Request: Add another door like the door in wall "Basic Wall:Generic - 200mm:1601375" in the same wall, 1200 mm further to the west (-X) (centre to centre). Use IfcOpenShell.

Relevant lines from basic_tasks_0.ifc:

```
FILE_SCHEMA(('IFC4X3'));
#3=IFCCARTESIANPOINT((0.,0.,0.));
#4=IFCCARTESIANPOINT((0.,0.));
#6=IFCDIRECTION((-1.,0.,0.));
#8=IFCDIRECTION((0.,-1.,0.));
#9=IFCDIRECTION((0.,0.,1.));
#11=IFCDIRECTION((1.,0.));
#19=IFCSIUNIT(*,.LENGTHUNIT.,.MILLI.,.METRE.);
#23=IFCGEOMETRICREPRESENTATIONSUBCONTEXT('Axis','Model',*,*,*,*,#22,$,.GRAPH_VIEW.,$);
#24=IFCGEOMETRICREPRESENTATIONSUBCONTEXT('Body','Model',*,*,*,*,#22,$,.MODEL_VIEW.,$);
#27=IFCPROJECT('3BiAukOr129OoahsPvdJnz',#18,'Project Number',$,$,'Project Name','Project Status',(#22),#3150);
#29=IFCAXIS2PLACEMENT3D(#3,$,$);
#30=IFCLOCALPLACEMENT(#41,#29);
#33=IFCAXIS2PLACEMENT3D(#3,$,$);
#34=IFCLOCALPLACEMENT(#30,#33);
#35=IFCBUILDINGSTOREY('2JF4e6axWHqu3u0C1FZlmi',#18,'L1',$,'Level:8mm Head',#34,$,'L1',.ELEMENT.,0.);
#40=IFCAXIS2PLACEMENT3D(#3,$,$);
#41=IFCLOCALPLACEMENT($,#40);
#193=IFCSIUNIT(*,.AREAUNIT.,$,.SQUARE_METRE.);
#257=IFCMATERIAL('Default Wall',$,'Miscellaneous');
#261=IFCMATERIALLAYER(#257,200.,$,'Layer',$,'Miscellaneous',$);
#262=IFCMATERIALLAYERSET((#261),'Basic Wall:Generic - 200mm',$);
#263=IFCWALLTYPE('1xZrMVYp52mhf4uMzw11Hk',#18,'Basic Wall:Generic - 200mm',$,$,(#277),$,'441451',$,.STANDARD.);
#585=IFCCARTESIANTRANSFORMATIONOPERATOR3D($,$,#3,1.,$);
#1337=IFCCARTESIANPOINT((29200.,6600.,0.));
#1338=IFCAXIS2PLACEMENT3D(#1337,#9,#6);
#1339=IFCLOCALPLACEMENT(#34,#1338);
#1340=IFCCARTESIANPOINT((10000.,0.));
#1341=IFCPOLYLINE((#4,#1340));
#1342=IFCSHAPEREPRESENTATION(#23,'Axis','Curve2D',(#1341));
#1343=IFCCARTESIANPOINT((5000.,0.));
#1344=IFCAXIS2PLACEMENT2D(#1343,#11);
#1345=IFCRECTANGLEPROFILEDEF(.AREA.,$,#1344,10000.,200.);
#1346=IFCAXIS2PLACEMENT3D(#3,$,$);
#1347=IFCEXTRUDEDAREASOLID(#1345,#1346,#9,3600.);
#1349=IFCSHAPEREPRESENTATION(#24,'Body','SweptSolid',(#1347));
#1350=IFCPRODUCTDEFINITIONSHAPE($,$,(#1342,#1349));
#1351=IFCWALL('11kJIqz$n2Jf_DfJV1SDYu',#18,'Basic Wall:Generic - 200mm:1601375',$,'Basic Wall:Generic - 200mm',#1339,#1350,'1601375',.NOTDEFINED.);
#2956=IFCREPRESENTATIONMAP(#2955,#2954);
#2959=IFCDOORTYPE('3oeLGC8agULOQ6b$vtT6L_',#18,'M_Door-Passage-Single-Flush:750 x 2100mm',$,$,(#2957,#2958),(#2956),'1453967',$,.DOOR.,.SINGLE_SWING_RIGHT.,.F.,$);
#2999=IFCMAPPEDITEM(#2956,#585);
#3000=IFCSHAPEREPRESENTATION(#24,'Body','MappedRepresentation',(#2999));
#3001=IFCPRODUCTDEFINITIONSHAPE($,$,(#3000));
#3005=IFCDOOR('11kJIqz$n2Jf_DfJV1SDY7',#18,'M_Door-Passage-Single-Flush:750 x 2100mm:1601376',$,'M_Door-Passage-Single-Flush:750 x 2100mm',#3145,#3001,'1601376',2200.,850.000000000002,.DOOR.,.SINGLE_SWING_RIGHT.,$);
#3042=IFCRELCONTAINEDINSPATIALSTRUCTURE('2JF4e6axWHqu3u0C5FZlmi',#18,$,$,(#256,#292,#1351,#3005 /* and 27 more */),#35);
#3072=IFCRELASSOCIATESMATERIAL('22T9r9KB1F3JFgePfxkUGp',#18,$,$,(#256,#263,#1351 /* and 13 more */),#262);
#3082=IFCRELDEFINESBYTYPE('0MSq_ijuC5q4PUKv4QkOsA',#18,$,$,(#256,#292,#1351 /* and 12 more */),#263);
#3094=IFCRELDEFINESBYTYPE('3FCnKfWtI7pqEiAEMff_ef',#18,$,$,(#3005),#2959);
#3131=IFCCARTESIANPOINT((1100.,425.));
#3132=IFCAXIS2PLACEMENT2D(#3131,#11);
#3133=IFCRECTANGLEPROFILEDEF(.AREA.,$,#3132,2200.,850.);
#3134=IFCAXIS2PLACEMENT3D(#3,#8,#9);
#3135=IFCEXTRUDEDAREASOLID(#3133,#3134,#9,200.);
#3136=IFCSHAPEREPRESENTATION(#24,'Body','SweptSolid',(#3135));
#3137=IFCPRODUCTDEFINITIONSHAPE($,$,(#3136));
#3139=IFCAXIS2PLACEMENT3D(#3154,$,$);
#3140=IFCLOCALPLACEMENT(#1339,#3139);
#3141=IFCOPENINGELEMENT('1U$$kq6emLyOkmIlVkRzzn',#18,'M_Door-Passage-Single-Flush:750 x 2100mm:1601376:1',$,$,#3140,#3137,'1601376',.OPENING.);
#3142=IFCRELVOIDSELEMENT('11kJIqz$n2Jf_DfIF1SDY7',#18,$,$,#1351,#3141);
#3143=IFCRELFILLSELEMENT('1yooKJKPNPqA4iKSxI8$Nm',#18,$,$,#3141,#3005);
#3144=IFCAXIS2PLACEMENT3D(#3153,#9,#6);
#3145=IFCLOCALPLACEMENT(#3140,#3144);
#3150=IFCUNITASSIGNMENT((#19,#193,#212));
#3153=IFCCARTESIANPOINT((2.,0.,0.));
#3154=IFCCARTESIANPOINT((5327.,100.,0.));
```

```python
import ifcopenshell
import ifcopenshell.api.feature
import ifcopenshell.api.geometry
import ifcopenshell.api.root
import ifcopenshell.geom
import ifcopenshell.util.element
import ifcopenshell.util.placement
import ifcopenshell.util.shape

model = ifcopenshell.open("basic_tasks_0.ifc")
settings = ifcopenshell.geom.settings()


def volume(element):
    """Net volume in cubic metres, openings subtracted."""
    shape = ifcopenshell.geom.create_shape(settings, element)
    return ifcopenshell.util.shape.get_volume(shape.geometry)


def reuse_history(source, copy):
    """copy_class also copies each property set's owner history, people and application; keep the originals."""
    for rel in copy.IsDefinedBy:
        if rel.is_a("IfcRelDefinesByProperties") and (history := rel.RelatingPropertyDefinition.OwnerHistory):
            rel.RelatingPropertyDefinition.OwnerHistory = source.OwnerHistory
            ifcopenshell.util.element.remove_deep2(model, history)


door = model.by_id(3005)
opening = door.FillsVoids[0].RelatingOpeningElement
wall = opening.VoidsElements[0].RelatingBuildingElement
before = volume(wall)
shift = ifcopenshell.util.placement.get_local_placement(wall.ObjectPlacement)[:3, 0] * 1200.0

# copy_class copies the void relationship, type, container and properties, but no geometry.
new_opening = ifcopenshell.api.root.copy_class(model, product=opening)
new_opening.Representation = ifcopenshell.util.element.copy_deep(
    model, opening.Representation, exclude=["IfcGeometricRepresentationContext", "IfcRepresentationMap"]
)
new_opening.Name = "M_Door-Passage-Single-Flush:750 x 2100mm"
new_opening.Tag = None
new_door = ifcopenshell.api.root.copy_class(model, product=door)
new_door.Representation = ifcopenshell.util.element.copy_deep(
    model, door.Representation, exclude=["IfcGeometricRepresentationContext", "IfcRepresentationMap"]
)
new_door.Name = "M_Door-Passage-Single-Flush:750 x 2100mm"
new_door.Tag = None
reuse_history(door, new_door)
ifcopenshell.api.feature.add_filling(model, opening=new_opening, element=new_door)

for old, new in ((opening, new_opening), (door, new_door)):
    matrix = ifcopenshell.util.placement.get_local_placement(old.ObjectPlacement)
    matrix[:3, 3] += shift
    ifcopenshell.api.geometry.edit_object_placement(model, product=new, matrix=matrix, is_si=False)

after = volume(wall)

print(f"wall volume {before:.3f} -> {after:.3f} m3")

model.write("basic_tasks_0_rev.ifc")
```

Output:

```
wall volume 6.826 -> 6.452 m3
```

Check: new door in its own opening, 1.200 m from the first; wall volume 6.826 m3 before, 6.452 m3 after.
